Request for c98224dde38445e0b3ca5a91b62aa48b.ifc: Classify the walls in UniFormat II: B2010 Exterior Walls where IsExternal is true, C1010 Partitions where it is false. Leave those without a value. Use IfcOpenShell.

First a look at what the model holds.

```python
import ifcopenshell
import ifcopenshell.util.element

model = ifcopenshell.open("c98224dde38445e0b3ca5a91b62aa48b.ifc")
print(model.schema)
print("classifications:", [c.Name for c in model.by_type("IfcClassification")])
values = [ifcopenshell.util.element.get_pset(e, "Pset_WallCommon", "IsExternal") for e in model.by_type("IfcWall")]
for value in (True, False, None):
    print("IsExternal", value, values.count(value))
```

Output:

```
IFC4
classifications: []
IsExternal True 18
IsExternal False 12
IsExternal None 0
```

```python
import ifcopenshell
import ifcopenshell.api.classification
import ifcopenshell.util.element

model = ifcopenshell.open("c98224dde38445e0b3ca5a91b62aa48b.ifc")

system = ifcopenshell.api.classification.add_classification(model, classification="UniFormat II")

walls = model.by_type("IfcWall")
external = {e: ifcopenshell.util.element.get_pset(e, "Pset_WallCommon", "IsExternal") for e in walls}
for flag, code, name in ((True, "B2010", "Exterior Walls"), (False, "C1010", "Partitions")):
    products = [e for e in walls if external[e] is flag]
    ifcopenshell.api.classification.add_reference(
        model, products=products, classification=system, identification=code, name=name
    )
    print(code, len(products))

model.write("c98224dde38445e0b3ca5a91b62aa48b_v2.ifc")
```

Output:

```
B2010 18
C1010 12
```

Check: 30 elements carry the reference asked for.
